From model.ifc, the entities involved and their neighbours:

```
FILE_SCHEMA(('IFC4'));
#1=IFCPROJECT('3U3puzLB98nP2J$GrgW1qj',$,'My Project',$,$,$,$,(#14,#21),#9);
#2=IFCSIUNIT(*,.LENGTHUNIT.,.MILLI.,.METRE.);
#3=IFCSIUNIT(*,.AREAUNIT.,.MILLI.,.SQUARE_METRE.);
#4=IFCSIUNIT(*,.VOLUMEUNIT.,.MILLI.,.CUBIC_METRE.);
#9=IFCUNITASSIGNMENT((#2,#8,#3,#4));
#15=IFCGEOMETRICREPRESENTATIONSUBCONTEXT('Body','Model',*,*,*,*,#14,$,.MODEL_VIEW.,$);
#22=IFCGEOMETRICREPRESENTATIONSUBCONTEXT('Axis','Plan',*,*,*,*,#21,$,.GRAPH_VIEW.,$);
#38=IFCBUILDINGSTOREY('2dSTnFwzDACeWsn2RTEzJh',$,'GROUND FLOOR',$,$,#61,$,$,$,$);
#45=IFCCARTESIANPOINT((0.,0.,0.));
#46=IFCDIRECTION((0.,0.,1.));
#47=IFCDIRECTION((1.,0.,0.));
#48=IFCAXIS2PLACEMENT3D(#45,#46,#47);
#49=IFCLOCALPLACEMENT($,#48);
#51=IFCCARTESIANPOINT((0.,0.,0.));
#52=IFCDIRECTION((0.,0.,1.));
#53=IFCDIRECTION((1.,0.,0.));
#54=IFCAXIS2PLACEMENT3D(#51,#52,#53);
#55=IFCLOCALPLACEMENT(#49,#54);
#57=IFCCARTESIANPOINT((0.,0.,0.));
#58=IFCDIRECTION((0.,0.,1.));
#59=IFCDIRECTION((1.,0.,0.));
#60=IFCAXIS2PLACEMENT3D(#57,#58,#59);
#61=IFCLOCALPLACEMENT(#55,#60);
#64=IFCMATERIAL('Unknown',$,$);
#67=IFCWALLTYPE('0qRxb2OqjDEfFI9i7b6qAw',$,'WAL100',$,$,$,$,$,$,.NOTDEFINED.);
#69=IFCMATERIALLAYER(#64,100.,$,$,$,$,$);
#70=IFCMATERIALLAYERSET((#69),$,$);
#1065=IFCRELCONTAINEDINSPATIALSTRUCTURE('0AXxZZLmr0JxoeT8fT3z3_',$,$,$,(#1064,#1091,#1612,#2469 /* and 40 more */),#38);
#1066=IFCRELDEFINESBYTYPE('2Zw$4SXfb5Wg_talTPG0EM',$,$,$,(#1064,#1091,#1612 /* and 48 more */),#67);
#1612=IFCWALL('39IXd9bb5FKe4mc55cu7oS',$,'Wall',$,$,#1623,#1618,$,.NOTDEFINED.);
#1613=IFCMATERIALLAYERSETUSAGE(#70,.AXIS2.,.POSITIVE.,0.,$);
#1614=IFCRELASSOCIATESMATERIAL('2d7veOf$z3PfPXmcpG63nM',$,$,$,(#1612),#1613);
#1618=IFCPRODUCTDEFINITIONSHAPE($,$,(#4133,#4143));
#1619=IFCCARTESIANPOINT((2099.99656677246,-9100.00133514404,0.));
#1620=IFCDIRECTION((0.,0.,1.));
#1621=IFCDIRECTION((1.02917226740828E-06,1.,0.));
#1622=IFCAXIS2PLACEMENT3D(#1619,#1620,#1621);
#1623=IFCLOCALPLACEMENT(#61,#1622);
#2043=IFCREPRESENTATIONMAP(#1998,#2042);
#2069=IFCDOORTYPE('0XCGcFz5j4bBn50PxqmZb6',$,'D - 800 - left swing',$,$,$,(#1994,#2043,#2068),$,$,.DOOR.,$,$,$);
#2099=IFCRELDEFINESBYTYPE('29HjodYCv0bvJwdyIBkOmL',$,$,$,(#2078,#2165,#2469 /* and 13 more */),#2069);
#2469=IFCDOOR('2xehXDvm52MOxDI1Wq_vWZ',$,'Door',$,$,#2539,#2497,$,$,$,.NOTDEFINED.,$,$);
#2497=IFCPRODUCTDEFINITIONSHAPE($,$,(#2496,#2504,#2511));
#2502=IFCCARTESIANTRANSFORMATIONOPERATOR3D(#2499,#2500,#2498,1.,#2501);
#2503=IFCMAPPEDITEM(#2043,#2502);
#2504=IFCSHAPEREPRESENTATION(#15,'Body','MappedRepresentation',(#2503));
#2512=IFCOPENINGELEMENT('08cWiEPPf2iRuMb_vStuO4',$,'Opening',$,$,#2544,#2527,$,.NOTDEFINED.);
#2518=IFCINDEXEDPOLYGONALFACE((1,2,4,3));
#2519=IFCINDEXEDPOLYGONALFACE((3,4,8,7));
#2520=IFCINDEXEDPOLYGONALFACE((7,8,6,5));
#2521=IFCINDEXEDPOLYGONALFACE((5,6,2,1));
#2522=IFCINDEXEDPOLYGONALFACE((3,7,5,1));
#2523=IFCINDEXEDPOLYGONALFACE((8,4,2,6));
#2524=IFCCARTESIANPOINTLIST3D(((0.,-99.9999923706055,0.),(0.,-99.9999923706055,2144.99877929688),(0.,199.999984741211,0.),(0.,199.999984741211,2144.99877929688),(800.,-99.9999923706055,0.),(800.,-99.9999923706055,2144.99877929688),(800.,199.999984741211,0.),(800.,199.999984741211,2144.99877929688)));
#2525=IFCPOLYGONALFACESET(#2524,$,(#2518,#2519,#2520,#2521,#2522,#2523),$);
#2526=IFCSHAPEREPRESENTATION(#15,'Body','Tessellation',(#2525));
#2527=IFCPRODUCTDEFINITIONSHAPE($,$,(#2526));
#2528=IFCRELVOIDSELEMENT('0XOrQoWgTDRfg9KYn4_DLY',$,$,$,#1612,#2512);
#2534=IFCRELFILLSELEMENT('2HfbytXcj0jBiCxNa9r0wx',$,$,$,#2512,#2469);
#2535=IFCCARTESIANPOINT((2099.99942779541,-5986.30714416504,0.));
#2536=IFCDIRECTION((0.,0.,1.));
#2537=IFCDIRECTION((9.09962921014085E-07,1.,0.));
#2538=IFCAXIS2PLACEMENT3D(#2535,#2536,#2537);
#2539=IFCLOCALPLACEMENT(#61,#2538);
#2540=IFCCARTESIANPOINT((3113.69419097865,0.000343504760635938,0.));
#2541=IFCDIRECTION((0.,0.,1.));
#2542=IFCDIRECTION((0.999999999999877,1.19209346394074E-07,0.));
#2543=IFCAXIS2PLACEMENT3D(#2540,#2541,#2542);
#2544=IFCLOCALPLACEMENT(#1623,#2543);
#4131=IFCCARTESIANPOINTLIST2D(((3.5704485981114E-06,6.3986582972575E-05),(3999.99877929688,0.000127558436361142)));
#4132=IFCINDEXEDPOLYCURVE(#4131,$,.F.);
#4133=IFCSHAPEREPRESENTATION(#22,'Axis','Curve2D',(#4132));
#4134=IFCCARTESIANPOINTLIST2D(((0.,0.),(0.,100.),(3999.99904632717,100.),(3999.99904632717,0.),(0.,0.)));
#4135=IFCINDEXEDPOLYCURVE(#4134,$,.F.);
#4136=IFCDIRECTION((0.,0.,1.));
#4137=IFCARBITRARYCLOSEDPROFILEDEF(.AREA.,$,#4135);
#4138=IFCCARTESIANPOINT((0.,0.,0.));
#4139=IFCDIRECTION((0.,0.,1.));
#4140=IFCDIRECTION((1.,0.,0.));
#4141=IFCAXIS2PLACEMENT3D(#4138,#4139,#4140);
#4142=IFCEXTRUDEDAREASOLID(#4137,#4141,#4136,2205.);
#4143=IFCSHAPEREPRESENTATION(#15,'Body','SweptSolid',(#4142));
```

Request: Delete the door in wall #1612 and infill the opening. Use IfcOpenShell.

```python
import ifcopenshell
import ifcopenshell.api.feature
import ifcopenshell.api.root
import ifcopenshell.geom
import ifcopenshell.util.shape

model = ifcopenshell.open("model.ifc")
settings = ifcopenshell.geom.settings()


def volume(element):
    """Net volume in cubic metres, openings subtracted."""
    shape = ifcopenshell.geom.create_shape(settings, element)
    return ifcopenshell.util.shape.get_volume(shape.geometry)


door = model.by_guid("2xehXDvm52MOxDI1Wq_vWZ")
opening = door.FillsVoids[0].RelatingOpeningElement
wall = opening.VoidsElements[0].RelatingBuildingElement
before = volume(wall)

ifcopenshell.api.root.remove_product(model, product=door)
ifcopenshell.api.feature.remove_feature(model, feature=opening)

after = volume(wall)

print(f"wall volume {before:.3f} -> {after:.3f} m3")

model.write("model_v2.ifc")
```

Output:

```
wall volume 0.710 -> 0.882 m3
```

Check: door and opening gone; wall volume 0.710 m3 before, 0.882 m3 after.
